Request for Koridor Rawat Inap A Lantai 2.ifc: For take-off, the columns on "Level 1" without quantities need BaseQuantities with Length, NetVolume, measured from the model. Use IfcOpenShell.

First a look at what the model holds.

```python
import ifcopenshell
import ifcopenshell.util.element
import ifcopenshell.util.unit

model = ifcopenshell.open("Koridor Rawat Inap A Lantai 2.ifc")
print(model.schema)
for unit_type in ("LENGTHUNIT", "AREAUNIT", "VOLUMEUNIT"):
    print(unit_type, ifcopenshell.util.unit.calculate_unit_scale(model, unit_type))
storey = next(s for s in model.by_type("IfcBuildingStorey") if s.Name == "Level 1")
columns = [e for e in ifcopenshell.util.element.get_decomposition(storey) if e.is_a("IfcColumn")]
for e in sorted(columns, key=lambda e: e.id()):
    print(e.id(), e.is_a(), e.Name, list(ifcopenshell.util.element.get_psets(e, qtos_only=True)), sep=" | ")
```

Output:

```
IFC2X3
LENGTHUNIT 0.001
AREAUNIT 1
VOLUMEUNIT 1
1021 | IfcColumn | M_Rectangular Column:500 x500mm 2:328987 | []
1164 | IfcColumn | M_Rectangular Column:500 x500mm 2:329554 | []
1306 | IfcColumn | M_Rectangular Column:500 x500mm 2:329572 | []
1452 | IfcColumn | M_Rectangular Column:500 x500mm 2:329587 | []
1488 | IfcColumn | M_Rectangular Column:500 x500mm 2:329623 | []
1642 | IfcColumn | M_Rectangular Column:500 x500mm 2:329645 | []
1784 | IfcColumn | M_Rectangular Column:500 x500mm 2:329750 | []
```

```python
import ifcopenshell
import ifcopenshell.api.pset
import ifcopenshell.geom
import ifcopenshell.util.element
import ifcopenshell.util.shape
import ifcopenshell.util.unit

model = ifcopenshell.open("Koridor Rawat Inap A Lantai 2.ifc")
unit_scale = ifcopenshell.util.unit.calculate_unit_scale(model)
volume_scale = ifcopenshell.util.unit.calculate_unit_scale(model, "VOLUMEUNIT")
settings = ifcopenshell.geom.settings()

storey = next(s for s in model.by_type("IfcBuildingStorey") if s.Name == "Level 1")
columns = [e for e in ifcopenshell.util.element.get_decomposition(storey) if e.is_a("IfcColumn")]

for e in sorted(columns, key=lambda e: e.id()):
    if ifcopenshell.util.element.get_psets(e, qtos_only=True, should_inherit=False):
        continue
    # Geometry comes back in metres, in the element's own axes.
    shape = ifcopenshell.geom.create_shape(settings, e)
    values = {
        "Length": ifcopenshell.util.shape.get_z(shape.geometry) / unit_scale,
        "NetVolume": ifcopenshell.util.shape.get_volume(shape.geometry) / volume_scale,
    }
    qto = ifcopenshell.api.pset.add_qto(model, product=e, name="BaseQuantities")
    ifcopenshell.api.pset.edit_qto(model, qto=qto, properties=values)
    print(e.id(), {k: round(v, 3) for k, v in values.items()})

model.write("Koridor Rawat Inap A Lantai 2_edited.ifc")
```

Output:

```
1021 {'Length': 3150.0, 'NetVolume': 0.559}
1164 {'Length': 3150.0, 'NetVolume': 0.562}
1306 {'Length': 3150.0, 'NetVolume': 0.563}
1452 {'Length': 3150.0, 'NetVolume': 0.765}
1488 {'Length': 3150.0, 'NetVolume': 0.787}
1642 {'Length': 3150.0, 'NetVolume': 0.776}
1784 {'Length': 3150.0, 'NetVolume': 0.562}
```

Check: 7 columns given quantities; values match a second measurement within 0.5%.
